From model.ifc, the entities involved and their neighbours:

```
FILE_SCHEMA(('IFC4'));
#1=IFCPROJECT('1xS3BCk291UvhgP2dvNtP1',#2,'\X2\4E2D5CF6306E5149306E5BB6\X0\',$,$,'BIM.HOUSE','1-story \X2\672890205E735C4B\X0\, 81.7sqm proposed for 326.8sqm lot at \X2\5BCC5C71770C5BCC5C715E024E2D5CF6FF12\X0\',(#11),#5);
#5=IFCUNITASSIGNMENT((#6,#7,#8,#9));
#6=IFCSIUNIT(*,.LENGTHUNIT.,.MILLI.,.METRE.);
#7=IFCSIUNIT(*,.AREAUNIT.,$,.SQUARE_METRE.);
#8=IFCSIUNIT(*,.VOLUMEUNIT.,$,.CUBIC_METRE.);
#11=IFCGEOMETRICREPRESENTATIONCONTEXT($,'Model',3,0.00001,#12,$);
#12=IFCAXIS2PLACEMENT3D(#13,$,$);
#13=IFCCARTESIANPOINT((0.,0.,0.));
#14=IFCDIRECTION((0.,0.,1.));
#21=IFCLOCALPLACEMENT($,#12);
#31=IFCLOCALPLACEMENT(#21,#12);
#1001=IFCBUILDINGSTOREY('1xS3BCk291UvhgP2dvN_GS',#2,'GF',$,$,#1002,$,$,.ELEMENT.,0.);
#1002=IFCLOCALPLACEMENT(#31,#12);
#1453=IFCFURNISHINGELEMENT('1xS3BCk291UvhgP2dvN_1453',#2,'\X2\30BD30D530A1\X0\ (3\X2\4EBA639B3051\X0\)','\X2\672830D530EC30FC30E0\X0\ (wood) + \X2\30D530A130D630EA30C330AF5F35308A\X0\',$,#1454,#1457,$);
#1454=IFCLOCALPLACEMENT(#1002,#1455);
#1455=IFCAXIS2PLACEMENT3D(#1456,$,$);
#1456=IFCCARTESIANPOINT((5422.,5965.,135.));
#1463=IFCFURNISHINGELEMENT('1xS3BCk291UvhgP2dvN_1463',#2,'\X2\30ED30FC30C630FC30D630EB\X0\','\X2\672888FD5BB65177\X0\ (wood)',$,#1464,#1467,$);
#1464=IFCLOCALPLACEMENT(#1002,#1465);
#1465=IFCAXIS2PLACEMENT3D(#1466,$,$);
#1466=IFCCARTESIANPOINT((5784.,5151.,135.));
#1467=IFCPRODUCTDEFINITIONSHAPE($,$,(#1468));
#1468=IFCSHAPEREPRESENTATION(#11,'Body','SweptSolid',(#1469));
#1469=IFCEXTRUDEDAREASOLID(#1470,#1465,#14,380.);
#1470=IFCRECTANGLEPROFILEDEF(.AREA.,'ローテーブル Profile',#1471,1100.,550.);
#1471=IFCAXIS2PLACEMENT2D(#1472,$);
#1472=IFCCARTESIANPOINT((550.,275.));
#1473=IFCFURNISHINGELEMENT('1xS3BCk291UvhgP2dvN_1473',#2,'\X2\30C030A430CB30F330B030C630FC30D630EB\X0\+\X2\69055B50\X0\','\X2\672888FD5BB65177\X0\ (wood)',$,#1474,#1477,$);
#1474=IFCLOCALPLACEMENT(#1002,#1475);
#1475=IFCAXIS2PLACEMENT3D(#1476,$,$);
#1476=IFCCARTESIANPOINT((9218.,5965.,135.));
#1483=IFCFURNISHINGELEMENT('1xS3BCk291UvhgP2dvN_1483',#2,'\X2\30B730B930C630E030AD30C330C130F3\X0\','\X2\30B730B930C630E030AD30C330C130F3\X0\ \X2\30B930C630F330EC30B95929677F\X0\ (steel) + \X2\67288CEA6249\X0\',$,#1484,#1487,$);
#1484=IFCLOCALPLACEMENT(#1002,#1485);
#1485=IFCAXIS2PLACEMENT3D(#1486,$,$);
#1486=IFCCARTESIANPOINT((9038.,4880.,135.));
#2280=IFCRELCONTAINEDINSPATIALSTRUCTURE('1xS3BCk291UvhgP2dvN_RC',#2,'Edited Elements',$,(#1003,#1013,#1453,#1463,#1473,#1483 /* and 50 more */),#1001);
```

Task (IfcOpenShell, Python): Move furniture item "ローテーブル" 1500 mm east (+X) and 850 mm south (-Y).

```python
import ifcopenshell
import ifcopenshell.api.geometry
import ifcopenshell.util.placement
import ifcopenshell.util.unit

model = ifcopenshell.open("model.ifc")
unit_scale = ifcopenshell.util.unit.calculate_unit_scale(model)

item = model.by_guid("1xS3BCk291UvhgP2dvN_1463")
matrix = ifcopenshell.util.placement.get_local_placement(item.ObjectPlacement)
matrix[0, 3] += 1.5 / unit_scale
matrix[1, 3] -= 0.85 / unit_scale
ifcopenshell.api.geometry.edit_object_placement(model, product=item, matrix=matrix, is_si=False)

print(ifcopenshell.util.placement.get_local_placement(item.ObjectPlacement).round(3) + 0.0)

model.write("model_v2.ifc")
```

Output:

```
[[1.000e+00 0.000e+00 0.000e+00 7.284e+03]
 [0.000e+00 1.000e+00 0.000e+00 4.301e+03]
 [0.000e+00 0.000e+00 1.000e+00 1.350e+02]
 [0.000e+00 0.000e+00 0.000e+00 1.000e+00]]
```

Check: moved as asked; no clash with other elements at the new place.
